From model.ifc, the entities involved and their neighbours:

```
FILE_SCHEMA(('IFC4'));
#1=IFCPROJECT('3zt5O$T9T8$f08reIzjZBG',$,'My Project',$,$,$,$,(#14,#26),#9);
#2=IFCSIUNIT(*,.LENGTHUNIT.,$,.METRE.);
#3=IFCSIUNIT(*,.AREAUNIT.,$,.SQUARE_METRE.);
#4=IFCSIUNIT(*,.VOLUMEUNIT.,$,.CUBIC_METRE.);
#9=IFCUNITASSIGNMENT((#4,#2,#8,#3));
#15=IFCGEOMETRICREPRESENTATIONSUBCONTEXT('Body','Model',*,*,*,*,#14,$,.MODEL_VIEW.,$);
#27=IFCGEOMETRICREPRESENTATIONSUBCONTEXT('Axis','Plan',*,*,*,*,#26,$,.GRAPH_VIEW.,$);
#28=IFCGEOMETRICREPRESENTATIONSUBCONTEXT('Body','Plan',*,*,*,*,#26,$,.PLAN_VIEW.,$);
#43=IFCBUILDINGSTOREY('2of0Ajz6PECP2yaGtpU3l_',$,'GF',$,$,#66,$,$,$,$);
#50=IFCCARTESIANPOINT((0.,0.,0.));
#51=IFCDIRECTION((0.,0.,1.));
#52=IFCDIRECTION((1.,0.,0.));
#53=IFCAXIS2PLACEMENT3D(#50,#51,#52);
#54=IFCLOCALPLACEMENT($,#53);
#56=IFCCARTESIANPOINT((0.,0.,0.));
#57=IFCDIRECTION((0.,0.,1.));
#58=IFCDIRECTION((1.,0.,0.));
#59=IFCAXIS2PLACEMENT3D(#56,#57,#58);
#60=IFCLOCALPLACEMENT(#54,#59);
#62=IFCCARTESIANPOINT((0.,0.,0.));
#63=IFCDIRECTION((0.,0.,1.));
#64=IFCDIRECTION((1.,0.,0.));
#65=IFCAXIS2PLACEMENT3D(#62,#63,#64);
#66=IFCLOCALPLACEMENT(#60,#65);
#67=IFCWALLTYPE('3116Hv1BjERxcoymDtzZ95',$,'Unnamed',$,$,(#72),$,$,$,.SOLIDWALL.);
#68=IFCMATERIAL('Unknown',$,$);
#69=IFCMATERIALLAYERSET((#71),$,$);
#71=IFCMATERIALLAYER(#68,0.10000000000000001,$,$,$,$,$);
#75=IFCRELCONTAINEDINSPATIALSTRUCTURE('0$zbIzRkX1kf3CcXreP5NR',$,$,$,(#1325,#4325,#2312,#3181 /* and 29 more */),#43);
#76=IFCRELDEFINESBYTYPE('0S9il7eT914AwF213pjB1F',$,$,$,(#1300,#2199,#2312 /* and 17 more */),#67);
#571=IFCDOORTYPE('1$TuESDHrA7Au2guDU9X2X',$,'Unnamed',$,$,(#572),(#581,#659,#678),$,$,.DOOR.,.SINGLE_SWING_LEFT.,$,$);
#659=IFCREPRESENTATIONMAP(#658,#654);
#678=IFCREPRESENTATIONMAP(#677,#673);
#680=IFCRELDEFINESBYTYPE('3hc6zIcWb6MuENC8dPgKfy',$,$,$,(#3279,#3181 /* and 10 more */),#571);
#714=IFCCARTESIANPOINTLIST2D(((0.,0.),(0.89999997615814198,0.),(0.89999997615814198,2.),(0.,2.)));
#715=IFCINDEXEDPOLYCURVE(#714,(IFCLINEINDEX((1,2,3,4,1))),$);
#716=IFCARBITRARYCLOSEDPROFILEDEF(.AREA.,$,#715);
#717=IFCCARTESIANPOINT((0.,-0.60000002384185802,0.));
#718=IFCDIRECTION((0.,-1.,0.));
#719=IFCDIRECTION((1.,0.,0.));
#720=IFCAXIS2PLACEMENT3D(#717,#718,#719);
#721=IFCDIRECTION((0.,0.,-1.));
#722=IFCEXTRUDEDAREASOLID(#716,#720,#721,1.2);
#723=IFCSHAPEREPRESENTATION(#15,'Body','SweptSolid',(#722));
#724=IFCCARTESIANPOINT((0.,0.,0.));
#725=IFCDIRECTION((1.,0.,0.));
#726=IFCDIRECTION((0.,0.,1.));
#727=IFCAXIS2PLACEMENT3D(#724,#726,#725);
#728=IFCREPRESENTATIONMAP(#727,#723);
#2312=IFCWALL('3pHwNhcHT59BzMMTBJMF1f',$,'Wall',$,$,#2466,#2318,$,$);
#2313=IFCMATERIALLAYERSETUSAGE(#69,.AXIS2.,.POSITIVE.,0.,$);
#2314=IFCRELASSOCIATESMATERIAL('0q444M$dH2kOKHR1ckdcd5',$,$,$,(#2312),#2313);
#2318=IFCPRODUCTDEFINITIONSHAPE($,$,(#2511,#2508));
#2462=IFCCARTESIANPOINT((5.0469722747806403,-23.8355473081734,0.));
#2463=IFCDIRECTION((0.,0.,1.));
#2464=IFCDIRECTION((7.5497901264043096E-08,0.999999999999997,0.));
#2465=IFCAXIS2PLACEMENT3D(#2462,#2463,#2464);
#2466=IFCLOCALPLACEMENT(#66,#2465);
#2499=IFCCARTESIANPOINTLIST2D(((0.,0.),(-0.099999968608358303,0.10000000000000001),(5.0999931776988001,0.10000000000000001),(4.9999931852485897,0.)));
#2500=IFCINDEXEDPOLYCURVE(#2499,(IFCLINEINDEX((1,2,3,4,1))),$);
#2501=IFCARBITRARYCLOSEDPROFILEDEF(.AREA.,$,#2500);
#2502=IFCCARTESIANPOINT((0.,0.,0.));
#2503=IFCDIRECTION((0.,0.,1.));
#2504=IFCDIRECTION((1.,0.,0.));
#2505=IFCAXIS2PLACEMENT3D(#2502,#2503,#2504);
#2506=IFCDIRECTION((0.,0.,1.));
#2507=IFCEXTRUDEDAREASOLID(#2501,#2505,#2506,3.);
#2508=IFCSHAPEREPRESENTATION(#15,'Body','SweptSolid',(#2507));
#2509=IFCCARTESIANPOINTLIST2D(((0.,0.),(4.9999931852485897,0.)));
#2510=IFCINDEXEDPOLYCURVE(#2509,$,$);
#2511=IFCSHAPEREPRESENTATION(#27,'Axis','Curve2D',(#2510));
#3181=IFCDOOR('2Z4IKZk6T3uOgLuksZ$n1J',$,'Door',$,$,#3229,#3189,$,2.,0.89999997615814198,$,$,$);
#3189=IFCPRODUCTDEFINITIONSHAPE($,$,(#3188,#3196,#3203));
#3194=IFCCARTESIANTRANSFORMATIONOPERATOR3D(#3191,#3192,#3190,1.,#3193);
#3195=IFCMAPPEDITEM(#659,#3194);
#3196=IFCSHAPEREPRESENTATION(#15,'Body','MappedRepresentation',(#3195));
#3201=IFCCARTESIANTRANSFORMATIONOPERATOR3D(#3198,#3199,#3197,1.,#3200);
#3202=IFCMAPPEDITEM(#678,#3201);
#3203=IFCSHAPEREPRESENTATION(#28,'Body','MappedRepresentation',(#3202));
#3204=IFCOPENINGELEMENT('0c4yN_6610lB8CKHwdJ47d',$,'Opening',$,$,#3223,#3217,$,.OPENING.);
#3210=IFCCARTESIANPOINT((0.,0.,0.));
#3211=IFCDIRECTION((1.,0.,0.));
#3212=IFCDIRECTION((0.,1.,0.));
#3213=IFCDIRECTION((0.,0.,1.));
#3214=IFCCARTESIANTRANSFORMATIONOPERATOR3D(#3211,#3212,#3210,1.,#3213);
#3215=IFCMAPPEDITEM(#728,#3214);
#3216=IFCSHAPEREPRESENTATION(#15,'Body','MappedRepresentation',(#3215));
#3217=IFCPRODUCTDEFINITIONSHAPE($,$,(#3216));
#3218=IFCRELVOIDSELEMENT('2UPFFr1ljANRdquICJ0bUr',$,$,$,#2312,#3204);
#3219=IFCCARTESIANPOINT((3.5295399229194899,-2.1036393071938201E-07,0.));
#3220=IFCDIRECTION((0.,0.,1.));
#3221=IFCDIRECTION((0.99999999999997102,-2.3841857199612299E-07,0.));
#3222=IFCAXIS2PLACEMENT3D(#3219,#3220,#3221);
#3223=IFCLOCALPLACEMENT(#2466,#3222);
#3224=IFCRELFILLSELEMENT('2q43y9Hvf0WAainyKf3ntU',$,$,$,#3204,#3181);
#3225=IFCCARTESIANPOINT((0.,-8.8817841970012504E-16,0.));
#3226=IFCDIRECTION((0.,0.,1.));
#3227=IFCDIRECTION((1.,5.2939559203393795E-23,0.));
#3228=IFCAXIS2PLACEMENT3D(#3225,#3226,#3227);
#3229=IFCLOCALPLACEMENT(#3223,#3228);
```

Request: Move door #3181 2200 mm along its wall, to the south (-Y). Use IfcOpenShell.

```python
import ifcopenshell
import ifcopenshell.api.geometry
import ifcopenshell.util.placement

model = ifcopenshell.open("model.ifc")

door = model.by_guid("2Z4IKZk6T3uOgLuksZ$n1J")
opening = door.FillsVoids[0].RelatingOpeningElement
wall = opening.VoidsElements[0].RelatingBuildingElement

wall_matrix = ifcopenshell.util.placement.get_local_placement(wall.ObjectPlacement)
shift = wall_matrix[:3, 0] * -2.2
before = ifcopenshell.util.placement.get_local_placement(door.ObjectPlacement)[:3, 3].copy()

# The door is placed relative to its opening, so it follows when the opening moves.
matrix = ifcopenshell.util.placement.get_local_placement(opening.ObjectPlacement)
matrix[:3, 3] += shift
ifcopenshell.api.geometry.edit_object_placement(
    model, product=opening, matrix=matrix, is_si=False, should_transform_children=True
)

after = ifcopenshell.util.placement.get_local_placement(door.ObjectPlacement)[:3, 3]
print("door moved by", (after - before).round(3) + 0.0)

model.write("model_rev.ifc")
```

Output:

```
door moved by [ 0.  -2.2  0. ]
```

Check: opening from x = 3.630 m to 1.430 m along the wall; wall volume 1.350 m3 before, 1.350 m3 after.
